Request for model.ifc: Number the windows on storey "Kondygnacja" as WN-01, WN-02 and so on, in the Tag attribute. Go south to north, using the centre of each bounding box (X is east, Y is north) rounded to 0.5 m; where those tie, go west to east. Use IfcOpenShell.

First a look at what the model holds.

```python
import ifcopenshell
import ifcopenshell.util.element
import ifcopenshell.util.placement

model = ifcopenshell.open("model.ifc")
print(model.schema)
storey = next(s for s in model.by_type("IfcBuildingStorey") if s.Name == "Kondygnacja")
windows = [e for e in ifcopenshell.util.element.get_decomposition(storey) if e.is_a("IfcWindow")]
for e in sorted(windows, key=lambda e: e.id()):
    origin = ifcopenshell.util.placement.get_local_placement(e.ObjectPlacement)[:3, 3]
    print(e.id(), e.Tag, e.Name, origin.round(2) + 0.0, sep=" | ")
```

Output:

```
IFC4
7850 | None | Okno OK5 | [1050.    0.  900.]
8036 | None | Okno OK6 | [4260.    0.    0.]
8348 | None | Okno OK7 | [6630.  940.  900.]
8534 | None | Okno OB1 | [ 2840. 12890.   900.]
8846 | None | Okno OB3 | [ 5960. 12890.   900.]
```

```python
import ifcopenshell
import ifcopenshell.geom
import ifcopenshell.util.element
import ifcopenshell.util.shape

model = ifcopenshell.open("model.ifc")
settings = ifcopenshell.geom.settings()
settings.set("use-world-coords", True)


def centre(element):
    shape = ifcopenshell.geom.create_shape(settings, element)
    return ifcopenshell.util.shape.get_bbox_centroid(shape.geometry)


storey = next(s for s in model.by_type("IfcBuildingStorey") if s.Name == "Kondygnacja")
windows = [e for e in ifcopenshell.util.element.get_decomposition(storey) if e.is_a("IfcWindow")]

# Insertion points can sit at a corner or the storey origin, so sort by the geometry (in metres).
centres = {e: centre(e) for e in windows}
windows.sort(key=lambda e: (round(centres[e][1] / 0.5), centres[e][0]))

for i, e in enumerate(windows, start=1):
    number = f"WN-{i:02d}"
    e.Tag = number
    print(e.id(), number)

model.write("model_edited.ifc")
```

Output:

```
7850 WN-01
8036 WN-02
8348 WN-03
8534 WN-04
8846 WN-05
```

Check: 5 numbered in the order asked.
